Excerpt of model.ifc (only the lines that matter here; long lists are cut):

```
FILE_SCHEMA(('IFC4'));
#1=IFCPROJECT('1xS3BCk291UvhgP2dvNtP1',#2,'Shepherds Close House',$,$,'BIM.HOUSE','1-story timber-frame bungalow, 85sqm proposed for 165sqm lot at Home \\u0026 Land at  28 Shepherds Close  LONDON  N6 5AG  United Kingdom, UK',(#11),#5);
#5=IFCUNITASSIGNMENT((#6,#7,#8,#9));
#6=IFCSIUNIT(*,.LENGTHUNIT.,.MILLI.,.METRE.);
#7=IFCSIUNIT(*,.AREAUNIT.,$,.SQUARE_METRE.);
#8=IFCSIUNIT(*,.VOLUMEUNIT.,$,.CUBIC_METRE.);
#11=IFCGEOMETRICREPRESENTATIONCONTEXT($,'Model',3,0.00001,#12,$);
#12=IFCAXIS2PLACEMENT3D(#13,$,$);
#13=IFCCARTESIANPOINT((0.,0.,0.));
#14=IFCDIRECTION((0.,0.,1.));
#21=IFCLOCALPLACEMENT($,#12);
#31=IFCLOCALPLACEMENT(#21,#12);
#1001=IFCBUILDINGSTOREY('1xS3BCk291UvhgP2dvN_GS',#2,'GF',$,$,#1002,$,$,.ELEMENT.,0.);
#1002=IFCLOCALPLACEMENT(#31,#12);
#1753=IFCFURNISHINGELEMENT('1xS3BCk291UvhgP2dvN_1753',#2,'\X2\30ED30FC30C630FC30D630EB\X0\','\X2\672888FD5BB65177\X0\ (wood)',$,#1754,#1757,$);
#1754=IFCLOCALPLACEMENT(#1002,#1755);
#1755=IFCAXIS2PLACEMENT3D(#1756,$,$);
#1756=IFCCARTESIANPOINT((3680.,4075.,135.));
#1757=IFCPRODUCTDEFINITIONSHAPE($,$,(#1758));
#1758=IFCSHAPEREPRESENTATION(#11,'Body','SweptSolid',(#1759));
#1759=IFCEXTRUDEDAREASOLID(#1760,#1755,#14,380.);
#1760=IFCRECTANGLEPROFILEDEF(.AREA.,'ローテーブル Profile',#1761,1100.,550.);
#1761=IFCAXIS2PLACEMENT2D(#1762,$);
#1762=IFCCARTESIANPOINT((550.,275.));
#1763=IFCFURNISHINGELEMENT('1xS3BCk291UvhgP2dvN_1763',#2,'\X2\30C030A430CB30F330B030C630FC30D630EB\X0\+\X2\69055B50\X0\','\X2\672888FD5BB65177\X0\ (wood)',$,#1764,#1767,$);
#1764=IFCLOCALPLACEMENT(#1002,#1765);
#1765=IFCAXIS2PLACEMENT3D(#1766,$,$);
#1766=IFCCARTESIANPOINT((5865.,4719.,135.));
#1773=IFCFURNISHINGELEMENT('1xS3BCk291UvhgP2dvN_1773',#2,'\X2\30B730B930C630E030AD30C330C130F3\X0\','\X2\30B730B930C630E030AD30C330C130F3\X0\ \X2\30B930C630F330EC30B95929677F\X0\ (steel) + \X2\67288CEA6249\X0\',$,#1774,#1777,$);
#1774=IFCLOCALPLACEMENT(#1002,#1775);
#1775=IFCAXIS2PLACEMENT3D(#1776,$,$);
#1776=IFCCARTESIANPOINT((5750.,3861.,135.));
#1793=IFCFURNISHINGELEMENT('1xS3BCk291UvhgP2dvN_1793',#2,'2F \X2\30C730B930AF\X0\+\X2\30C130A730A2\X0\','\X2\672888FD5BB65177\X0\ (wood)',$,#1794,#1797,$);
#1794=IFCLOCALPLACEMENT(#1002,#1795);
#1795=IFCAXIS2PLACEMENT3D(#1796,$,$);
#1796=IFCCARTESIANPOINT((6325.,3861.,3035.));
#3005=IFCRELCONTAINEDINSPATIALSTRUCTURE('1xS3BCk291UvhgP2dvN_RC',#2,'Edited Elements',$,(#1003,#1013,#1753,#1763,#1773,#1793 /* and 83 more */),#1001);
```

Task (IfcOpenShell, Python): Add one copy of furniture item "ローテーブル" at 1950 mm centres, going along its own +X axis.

```python
import ifcopenshell
import ifcopenshell.api.geometry
import ifcopenshell.api.root
import ifcopenshell.util.element
import ifcopenshell.util.placement

model = ifcopenshell.open("model.ifc")


def reuse_history(source, copy):
    """copy_class also copies each property set's owner history, people and application; keep the originals."""
    for rel in copy.IsDefinedBy:
        if rel.is_a("IfcRelDefinesByProperties") and (history := rel.RelatingPropertyDefinition.OwnerHistory):
            rel.RelatingPropertyDefinition.OwnerHistory = source.OwnerHistory
            ifcopenshell.util.element.remove_deep2(model, history)


source = model.by_guid("1xS3BCk291UvhgP2dvN_1753")
base = ifcopenshell.util.placement.get_local_placement(source.ObjectPlacement)
step = base[:3, 0] * 1950.0

for i in range(1, 2):
    copy = ifcopenshell.api.root.copy_class(model, product=source)
    copy.Representation = ifcopenshell.util.element.copy_deep(
        model, source.Representation, exclude=["IfcGeometricRepresentationContext", "IfcRepresentationMap"]
    )
    reuse_history(source, copy)
    matrix = base.copy()
    matrix[:3, 3] += i * step
    print("added at", matrix[:3, 3].round(3) + 0.0)
    ifcopenshell.api.geometry.edit_object_placement(model, product=copy, matrix=matrix, is_si=False)

model.write("model-out.ifc")
```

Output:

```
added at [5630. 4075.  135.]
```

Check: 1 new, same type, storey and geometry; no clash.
